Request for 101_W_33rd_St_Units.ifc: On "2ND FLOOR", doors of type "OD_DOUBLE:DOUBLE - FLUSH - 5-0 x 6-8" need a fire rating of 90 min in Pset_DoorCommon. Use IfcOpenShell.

First a look at what the model holds.

```python
import ifcopenshell
import ifcopenshell.util.element

model = ifcopenshell.open("101_W_33rd_St_Units.ifc")
print(model.schema)
storey = next(s for s in model.by_type("IfcBuildingStorey") if s.Name == "2ND FLOOR")
doors = [e for e in ifcopenshell.util.element.get_decomposition(storey) if e.is_a("IfcDoor")]
seen = {}
for e in doors:
    element_type = ifcopenshell.util.element.get_type(e)
    key = (element_type.Name if element_type != e and element_type else None, ifcopenshell.util.element.get_pset(e, "Pset_DoorCommon", "FireRating"))
    seen[key] = seen.get(key, 0) + 1
for (name, value), count in sorted(seen.items(), key=str):
    print(count, "x", name, "|", value)
```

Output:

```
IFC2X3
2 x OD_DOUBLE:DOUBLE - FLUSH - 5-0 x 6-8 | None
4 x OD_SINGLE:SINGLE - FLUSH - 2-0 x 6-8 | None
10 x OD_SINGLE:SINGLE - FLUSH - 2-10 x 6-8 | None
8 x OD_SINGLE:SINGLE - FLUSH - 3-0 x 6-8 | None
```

```python
import ifcopenshell
import ifcopenshell.api.pset
import ifcopenshell.util.element

model = ifcopenshell.open("101_W_33rd_St_Units.ifc")

storey = next(s for s in model.by_type("IfcBuildingStorey") if s.Name == "2ND FLOOR")
doors = [e for e in ifcopenshell.util.element.get_decomposition(storey) if e.is_a("IfcDoor")]

count = 0
for e in doors:
    element_type = ifcopenshell.util.element.get_type(e)
    if element_type in (None, e) or element_type.Name != "OD_DOUBLE:DOUBLE - FLUSH - 5-0 x 6-8":
        continue
    # add_pset returns the element's existing set when there is one.
    pset = ifcopenshell.api.pset.add_pset(model, product=e, name="Pset_DoorCommon")
    ifcopenshell.api.pset.edit_pset(model, pset=pset, properties={"FireRating": "90 min"})
    count += 1

print(count, "doors updated")

model.write("101_W_33rd_St_Units_v2.ifc")
```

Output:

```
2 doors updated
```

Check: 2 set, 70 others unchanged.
